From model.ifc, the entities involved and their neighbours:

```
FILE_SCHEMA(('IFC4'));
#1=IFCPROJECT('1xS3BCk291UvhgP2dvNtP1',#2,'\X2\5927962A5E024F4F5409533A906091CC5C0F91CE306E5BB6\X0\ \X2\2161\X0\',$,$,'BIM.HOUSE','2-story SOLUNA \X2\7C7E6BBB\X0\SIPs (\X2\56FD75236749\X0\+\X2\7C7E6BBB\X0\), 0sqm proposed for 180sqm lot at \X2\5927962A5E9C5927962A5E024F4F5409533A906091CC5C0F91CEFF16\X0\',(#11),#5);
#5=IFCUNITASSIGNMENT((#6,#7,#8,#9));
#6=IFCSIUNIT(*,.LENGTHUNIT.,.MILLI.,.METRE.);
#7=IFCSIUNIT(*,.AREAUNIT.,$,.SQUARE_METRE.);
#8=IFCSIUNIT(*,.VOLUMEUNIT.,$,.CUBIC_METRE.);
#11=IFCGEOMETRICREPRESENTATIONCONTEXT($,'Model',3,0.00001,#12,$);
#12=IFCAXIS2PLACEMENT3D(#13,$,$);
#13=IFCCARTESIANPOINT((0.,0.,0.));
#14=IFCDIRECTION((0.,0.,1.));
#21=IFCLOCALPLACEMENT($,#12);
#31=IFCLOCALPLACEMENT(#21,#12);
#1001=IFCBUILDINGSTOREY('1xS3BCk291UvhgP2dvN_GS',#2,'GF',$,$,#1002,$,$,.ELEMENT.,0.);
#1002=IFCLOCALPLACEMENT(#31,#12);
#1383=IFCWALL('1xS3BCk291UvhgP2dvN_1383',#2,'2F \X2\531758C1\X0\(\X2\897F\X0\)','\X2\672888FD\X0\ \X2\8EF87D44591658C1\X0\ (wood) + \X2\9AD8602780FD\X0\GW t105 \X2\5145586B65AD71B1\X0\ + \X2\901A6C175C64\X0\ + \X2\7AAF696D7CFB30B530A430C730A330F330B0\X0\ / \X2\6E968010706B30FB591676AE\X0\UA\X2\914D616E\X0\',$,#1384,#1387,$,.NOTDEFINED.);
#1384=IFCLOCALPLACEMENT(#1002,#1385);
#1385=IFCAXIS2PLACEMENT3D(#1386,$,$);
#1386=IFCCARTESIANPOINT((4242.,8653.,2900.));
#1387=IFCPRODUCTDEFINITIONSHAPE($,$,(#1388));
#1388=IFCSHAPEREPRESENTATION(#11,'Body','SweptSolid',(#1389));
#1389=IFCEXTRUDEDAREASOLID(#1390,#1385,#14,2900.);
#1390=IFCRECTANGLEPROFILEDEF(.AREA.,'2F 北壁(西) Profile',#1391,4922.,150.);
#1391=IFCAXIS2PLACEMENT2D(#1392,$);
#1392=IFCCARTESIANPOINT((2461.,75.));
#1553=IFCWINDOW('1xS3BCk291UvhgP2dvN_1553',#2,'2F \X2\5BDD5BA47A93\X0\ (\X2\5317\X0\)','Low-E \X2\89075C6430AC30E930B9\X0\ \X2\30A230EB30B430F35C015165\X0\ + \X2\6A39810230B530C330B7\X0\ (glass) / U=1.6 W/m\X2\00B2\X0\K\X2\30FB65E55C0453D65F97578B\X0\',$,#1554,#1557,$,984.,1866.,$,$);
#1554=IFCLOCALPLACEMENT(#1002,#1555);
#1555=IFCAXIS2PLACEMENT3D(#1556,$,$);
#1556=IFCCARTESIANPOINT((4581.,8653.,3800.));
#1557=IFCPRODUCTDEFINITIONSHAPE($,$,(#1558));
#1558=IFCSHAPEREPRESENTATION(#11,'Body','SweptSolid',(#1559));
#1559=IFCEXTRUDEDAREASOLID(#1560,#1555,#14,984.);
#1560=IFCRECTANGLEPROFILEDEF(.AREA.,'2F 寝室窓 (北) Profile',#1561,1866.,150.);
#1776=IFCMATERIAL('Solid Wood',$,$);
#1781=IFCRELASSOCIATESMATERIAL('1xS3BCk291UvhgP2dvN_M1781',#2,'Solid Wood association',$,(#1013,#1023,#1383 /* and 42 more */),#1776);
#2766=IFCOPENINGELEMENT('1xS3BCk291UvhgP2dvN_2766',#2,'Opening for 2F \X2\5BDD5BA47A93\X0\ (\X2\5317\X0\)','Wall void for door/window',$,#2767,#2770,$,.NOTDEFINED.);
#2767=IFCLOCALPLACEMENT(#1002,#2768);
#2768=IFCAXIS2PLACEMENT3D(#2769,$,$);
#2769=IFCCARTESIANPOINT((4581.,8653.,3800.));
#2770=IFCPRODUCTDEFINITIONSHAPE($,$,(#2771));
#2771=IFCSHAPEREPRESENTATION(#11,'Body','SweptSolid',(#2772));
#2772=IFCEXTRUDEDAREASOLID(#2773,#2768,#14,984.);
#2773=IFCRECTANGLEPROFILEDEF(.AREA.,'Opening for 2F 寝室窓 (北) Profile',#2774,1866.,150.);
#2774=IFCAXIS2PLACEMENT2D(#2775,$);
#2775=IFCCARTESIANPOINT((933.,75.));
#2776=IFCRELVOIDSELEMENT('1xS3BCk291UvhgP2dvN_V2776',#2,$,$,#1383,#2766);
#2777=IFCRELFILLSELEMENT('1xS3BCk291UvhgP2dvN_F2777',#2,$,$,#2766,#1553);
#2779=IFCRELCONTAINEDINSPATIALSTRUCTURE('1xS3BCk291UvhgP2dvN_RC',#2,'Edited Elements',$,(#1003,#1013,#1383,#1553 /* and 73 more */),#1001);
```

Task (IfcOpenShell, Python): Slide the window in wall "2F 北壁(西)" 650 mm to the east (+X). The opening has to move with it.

```python
import ifcopenshell
import ifcopenshell.api.geometry
import ifcopenshell.util.placement

model = ifcopenshell.open("model.ifc")

window = model.by_guid("1xS3BCk291UvhgP2dvN_1553")
opening = window.FillsVoids[0].RelatingOpeningElement
wall = opening.VoidsElements[0].RelatingBuildingElement

wall_matrix = ifcopenshell.util.placement.get_local_placement(wall.ObjectPlacement)
shift = wall_matrix[:3, 0] * 650.0
before = ifcopenshell.util.placement.get_local_placement(window.ObjectPlacement)[:3, 3].copy()

# The window is not placed relative to its opening, so move both.
for product in (opening, window):
    matrix = ifcopenshell.util.placement.get_local_placement(product.ObjectPlacement)
    matrix[:3, 3] += shift
    ifcopenshell.api.geometry.edit_object_placement(model, product=product, matrix=matrix, is_si=False)

after = ifcopenshell.util.placement.get_local_placement(window.ObjectPlacement)[:3, 3]
print("window moved by", (after - before).round(3) + 0.0)

model.write("model_v2.ifc")
```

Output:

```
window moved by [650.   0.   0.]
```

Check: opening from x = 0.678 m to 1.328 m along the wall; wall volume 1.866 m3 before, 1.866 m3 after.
